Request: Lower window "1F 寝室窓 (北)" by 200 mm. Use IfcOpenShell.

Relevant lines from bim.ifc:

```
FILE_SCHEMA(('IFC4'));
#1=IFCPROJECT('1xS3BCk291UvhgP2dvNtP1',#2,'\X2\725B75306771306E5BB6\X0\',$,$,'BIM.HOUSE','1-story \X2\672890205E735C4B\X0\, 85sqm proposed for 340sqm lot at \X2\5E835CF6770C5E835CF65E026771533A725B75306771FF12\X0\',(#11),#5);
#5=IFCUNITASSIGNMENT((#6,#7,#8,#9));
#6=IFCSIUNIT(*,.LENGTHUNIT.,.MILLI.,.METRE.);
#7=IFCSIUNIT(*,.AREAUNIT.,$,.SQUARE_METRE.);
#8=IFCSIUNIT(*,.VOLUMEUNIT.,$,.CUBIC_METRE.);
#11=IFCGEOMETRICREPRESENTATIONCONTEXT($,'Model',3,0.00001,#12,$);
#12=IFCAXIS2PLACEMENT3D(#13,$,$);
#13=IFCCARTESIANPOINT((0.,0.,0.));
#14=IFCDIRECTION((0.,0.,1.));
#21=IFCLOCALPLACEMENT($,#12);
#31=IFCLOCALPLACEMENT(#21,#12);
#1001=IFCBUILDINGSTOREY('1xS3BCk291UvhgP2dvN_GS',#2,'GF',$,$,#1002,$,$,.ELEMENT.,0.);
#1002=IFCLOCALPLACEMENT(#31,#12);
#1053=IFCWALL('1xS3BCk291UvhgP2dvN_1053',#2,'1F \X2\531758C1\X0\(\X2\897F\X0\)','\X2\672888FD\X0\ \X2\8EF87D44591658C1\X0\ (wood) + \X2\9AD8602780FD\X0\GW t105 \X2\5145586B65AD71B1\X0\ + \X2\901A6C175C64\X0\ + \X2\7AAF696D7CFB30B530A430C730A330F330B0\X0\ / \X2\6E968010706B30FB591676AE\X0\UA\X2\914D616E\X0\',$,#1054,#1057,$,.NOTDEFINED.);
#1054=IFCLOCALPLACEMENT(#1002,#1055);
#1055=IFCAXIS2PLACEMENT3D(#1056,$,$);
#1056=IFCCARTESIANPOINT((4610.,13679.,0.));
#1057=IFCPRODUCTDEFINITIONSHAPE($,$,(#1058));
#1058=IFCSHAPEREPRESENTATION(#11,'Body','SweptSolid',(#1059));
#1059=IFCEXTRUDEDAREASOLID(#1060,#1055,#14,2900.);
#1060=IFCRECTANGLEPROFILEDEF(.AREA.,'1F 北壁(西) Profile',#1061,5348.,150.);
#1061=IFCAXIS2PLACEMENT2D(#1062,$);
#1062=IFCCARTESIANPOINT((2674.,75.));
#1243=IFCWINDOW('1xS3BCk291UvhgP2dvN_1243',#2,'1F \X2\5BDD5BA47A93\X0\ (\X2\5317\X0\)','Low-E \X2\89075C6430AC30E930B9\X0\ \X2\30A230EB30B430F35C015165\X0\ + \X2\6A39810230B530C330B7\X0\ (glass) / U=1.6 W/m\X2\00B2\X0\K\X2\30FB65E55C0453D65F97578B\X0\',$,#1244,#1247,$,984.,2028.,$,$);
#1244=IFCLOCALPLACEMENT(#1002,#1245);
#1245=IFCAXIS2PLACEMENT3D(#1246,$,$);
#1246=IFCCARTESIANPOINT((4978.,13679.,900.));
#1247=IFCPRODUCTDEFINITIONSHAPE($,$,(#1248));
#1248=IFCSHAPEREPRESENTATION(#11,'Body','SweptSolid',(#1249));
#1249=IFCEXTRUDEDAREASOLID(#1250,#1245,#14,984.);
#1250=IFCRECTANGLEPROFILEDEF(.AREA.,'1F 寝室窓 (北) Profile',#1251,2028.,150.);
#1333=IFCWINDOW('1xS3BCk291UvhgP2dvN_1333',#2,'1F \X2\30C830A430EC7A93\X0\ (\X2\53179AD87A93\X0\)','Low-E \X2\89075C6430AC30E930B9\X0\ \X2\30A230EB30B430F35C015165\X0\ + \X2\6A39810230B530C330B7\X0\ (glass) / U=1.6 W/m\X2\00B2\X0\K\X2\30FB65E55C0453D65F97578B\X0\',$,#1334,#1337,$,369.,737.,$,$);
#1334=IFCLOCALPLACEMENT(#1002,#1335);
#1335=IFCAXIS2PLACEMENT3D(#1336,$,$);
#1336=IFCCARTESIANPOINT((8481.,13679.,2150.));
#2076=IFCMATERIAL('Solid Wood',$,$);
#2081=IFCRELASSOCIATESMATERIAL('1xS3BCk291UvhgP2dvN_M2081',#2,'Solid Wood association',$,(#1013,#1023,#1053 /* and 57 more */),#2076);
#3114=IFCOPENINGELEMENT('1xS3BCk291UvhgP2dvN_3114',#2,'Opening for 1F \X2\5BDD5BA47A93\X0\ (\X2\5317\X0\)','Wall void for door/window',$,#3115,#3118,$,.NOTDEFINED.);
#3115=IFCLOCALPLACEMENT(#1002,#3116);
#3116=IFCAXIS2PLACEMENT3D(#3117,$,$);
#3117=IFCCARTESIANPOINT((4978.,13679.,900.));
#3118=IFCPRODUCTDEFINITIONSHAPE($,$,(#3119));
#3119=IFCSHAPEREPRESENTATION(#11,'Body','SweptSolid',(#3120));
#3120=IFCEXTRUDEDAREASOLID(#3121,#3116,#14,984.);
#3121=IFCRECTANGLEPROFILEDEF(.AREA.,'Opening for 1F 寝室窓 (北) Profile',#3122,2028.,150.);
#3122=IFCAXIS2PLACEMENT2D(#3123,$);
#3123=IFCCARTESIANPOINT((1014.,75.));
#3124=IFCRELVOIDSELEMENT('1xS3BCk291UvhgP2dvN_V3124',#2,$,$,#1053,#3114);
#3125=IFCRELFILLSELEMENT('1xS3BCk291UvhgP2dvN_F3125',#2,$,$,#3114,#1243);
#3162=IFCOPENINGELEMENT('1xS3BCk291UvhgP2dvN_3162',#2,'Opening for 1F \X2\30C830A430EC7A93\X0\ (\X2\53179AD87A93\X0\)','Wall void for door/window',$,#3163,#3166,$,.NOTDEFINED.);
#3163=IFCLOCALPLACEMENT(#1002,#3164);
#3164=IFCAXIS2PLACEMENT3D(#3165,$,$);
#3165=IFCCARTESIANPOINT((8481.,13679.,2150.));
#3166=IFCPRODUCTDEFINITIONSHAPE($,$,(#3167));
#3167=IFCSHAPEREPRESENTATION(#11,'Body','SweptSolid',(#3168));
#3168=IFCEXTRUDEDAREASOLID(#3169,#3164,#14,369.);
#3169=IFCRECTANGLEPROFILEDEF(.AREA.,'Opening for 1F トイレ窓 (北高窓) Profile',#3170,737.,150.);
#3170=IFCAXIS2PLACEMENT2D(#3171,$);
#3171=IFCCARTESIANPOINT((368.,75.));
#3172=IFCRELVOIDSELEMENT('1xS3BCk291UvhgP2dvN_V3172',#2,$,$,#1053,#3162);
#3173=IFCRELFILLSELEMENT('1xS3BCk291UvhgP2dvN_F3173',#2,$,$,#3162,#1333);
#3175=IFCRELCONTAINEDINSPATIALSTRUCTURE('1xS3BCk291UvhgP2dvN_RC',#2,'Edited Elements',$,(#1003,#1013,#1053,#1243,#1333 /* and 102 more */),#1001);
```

```python
import numpy as np
import ifcopenshell
import ifcopenshell.api.geometry
import ifcopenshell.util.placement
import ifcopenshell.util.unit

model = ifcopenshell.open("bim.ifc")
unit_scale = ifcopenshell.util.unit.calculate_unit_scale(model)

window = model.by_guid("1xS3BCk291UvhgP2dvN_1243")
opening = window.FillsVoids[0].RelatingOpeningElement
dz = -200.0

shift = np.array([0.0, 0.0, dz])
# The window is not placed relative to its opening, so move both.
for product in (opening, window):
    matrix = ifcopenshell.util.placement.get_local_placement(product.ObjectPlacement)
    matrix[:3, 3] += shift
    ifcopenshell.api.geometry.edit_object_placement(model, product=product, matrix=matrix, is_si=False)

print(f"moved by {dz * unit_scale:+.3f} m")

model.write("bim-out.ifc")
```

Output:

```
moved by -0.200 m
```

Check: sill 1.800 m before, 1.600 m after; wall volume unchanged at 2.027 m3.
